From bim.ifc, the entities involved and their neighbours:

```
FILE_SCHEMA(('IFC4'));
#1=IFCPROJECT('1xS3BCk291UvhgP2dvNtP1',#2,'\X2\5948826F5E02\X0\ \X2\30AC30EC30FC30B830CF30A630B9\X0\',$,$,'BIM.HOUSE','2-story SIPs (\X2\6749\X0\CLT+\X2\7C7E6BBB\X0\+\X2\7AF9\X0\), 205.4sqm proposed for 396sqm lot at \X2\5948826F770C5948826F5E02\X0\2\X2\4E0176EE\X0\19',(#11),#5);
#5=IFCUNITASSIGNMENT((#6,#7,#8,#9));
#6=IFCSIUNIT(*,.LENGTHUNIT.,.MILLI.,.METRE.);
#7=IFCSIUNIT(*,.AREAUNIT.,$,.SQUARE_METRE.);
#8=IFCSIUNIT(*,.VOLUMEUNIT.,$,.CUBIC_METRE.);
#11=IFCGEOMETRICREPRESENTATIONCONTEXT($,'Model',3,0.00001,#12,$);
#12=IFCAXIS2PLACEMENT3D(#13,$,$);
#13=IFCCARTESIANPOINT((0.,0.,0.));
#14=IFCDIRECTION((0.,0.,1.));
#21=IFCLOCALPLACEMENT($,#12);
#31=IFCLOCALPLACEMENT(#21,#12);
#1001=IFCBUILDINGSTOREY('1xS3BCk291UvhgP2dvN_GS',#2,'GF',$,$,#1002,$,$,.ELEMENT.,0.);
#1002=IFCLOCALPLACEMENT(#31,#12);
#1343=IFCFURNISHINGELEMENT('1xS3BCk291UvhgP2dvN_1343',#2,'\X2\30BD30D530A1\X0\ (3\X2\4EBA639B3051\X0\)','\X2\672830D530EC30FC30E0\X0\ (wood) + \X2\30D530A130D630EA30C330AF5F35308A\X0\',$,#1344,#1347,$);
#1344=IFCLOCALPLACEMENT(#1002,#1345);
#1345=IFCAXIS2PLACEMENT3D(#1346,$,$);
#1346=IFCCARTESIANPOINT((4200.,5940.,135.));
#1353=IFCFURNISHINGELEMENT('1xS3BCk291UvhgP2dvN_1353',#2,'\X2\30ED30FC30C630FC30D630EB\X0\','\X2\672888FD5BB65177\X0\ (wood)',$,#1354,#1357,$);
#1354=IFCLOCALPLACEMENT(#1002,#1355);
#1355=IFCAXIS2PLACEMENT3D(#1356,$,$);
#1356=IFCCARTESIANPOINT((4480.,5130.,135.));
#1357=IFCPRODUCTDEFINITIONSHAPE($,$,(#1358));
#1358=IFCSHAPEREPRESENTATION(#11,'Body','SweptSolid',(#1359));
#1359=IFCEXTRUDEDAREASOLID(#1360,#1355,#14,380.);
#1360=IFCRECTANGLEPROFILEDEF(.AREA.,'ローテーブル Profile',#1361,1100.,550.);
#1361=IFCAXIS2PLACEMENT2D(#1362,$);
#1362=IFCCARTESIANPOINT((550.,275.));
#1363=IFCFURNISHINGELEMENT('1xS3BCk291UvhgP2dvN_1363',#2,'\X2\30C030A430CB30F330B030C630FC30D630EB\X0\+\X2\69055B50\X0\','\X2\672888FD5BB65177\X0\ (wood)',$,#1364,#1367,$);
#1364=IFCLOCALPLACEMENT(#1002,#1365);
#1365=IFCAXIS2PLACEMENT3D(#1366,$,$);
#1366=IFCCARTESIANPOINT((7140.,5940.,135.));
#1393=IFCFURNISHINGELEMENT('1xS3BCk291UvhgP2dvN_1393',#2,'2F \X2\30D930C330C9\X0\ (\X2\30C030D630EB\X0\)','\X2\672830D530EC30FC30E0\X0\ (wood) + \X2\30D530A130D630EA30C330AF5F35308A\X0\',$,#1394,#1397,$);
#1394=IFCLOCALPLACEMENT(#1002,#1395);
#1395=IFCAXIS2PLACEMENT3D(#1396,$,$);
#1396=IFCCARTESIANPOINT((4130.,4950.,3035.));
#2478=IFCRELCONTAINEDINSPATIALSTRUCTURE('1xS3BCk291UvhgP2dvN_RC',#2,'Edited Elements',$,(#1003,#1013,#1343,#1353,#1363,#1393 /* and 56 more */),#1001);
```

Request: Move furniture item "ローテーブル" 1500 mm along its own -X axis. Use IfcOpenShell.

```python
import ifcopenshell
import ifcopenshell.api.geometry
import ifcopenshell.util.placement
import ifcopenshell.util.unit

model = ifcopenshell.open("bim.ifc")
unit_scale = ifcopenshell.util.unit.calculate_unit_scale(model)

item = model.by_guid("1xS3BCk291UvhgP2dvN_1353")
matrix = ifcopenshell.util.placement.get_local_placement(item.ObjectPlacement)
matrix[:3, 3] -= matrix[:3, 0] * 1.5 / unit_scale
ifcopenshell.api.geometry.edit_object_placement(model, product=item, matrix=matrix, is_si=False)

print(ifcopenshell.util.placement.get_local_placement(item.ObjectPlacement).round(3) + 0.0)

model.write("bim_edited.ifc")
```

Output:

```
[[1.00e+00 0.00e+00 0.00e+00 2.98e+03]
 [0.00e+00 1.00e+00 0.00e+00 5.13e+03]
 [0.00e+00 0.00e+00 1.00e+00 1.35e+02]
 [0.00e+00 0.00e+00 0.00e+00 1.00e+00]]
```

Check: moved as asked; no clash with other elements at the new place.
